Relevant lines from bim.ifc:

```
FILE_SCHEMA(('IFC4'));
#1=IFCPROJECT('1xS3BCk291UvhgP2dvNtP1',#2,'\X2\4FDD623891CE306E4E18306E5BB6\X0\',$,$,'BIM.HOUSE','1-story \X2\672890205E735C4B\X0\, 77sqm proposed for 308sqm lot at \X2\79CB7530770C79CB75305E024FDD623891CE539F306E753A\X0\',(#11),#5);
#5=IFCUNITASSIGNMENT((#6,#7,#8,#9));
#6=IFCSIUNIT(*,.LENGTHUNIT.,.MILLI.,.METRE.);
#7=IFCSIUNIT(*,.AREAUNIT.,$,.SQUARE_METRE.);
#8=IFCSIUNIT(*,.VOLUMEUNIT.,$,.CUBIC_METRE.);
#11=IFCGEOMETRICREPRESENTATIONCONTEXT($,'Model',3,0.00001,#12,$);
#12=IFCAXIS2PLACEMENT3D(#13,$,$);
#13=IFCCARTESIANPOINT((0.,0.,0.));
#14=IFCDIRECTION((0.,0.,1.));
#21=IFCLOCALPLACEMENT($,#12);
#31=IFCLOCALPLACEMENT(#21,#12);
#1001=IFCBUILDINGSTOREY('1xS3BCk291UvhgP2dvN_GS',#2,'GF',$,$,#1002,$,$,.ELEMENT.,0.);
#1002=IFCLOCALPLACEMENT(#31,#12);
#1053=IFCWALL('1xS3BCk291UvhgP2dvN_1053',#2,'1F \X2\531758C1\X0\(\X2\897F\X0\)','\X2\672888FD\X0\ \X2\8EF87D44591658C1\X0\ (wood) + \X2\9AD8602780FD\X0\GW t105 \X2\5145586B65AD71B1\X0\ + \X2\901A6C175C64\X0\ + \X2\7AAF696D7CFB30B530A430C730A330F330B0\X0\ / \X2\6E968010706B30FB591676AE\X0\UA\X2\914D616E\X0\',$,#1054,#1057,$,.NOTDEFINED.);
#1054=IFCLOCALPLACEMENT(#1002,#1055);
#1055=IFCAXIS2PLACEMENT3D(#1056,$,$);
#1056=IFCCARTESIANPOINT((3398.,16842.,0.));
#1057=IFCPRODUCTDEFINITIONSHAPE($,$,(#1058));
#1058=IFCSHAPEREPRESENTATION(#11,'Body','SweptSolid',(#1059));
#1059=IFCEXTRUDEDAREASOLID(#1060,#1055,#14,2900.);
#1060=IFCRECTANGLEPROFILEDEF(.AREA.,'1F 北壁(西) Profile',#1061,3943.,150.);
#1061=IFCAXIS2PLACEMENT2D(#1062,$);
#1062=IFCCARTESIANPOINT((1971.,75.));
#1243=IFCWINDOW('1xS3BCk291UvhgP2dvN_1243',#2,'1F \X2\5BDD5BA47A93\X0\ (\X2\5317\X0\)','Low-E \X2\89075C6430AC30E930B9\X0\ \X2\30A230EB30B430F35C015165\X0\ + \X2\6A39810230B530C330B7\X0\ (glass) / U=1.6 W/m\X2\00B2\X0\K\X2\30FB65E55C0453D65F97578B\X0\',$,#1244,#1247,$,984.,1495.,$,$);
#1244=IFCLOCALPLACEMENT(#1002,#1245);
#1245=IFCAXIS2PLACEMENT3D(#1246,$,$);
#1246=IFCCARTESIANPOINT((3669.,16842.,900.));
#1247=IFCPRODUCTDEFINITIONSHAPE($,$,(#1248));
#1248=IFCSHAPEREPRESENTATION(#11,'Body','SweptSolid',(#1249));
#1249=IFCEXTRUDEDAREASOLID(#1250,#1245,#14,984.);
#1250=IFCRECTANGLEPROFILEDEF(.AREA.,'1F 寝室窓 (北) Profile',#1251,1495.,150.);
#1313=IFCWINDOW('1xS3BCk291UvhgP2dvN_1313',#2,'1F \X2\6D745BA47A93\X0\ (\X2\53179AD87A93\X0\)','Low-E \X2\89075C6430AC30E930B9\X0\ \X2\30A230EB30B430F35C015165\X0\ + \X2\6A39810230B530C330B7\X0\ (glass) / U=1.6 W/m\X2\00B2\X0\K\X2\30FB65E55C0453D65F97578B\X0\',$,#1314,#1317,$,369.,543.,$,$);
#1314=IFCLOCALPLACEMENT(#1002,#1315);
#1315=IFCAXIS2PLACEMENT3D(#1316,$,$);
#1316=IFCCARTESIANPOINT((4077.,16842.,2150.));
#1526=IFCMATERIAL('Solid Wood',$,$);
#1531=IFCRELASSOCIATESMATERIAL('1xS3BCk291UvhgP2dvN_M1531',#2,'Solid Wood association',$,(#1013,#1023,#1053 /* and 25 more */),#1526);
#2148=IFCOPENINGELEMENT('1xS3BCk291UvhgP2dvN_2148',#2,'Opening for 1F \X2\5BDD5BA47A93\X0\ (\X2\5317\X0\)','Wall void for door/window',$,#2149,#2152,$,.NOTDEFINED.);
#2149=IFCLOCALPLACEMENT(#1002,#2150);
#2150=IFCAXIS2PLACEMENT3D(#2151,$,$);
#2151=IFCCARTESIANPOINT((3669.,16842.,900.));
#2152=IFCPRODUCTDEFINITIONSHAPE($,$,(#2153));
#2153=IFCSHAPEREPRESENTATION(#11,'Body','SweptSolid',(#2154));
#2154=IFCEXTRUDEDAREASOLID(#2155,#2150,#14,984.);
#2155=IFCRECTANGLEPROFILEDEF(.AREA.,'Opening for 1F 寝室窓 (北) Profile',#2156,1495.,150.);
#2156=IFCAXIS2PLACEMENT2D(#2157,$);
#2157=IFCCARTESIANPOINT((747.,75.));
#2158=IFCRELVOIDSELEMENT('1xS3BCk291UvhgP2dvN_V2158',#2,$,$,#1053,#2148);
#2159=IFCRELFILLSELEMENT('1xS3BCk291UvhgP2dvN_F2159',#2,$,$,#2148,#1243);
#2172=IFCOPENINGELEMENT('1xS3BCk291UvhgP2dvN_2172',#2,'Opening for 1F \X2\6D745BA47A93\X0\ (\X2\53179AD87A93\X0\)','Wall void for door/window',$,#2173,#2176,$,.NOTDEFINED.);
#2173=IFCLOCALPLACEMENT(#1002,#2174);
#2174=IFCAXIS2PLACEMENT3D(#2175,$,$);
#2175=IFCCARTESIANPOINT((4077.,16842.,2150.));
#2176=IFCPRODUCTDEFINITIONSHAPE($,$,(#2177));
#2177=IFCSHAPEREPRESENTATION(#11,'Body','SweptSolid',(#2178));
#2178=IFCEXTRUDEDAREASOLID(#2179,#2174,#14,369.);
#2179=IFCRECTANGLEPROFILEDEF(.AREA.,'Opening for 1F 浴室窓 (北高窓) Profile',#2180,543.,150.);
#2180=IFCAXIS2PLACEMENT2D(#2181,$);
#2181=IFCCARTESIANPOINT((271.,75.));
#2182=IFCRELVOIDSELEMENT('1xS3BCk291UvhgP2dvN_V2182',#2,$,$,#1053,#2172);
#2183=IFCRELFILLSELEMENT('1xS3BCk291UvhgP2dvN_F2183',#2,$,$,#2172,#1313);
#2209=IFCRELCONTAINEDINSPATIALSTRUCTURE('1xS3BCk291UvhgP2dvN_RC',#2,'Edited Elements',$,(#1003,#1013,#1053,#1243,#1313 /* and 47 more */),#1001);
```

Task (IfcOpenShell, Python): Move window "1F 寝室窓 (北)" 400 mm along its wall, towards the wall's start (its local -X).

```python
import ifcopenshell
import ifcopenshell.api.geometry
import ifcopenshell.util.placement
import ifcopenshell.util.unit

model = ifcopenshell.open("bim.ifc")
unit_scale = ifcopenshell.util.unit.calculate_unit_scale(model)

window = model.by_guid("1xS3BCk291UvhgP2dvN_1243")
opening = window.FillsVoids[0].RelatingOpeningElement
wall = opening.VoidsElements[0].RelatingBuildingElement

wall_matrix = ifcopenshell.util.placement.get_local_placement(wall.ObjectPlacement)
shift = wall_matrix[:3, 0] * -0.4 / unit_scale
before = ifcopenshell.util.placement.get_local_placement(window.ObjectPlacement)[:3, 3].copy()

# The window is not placed relative to its opening, so move both.
for product in (opening, window):
    matrix = ifcopenshell.util.placement.get_local_placement(product.ObjectPlacement)
    matrix[:3, 3] += shift
    ifcopenshell.api.geometry.edit_object_placement(model, product=product, matrix=matrix, is_si=False)

after = ifcopenshell.util.placement.get_local_placement(window.ObjectPlacement)[:3, 3]
print("window moved by", (after - before).round(3) + 0.0)

model.write("bim_rev.ifc")
```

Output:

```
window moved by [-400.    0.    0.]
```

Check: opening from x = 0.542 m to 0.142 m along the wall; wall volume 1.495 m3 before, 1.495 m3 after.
